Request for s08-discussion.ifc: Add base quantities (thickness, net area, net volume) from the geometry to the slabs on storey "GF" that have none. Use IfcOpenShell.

First a look at what the model holds.

```python
import ifcopenshell
import ifcopenshell.util.element
import ifcopenshell.util.unit

model = ifcopenshell.open("s08-discussion.ifc")
print(model.schema)
for unit_type in ("LENGTHUNIT", "AREAUNIT", "VOLUMEUNIT"):
    print(unit_type, ifcopenshell.util.unit.calculate_unit_scale(model, unit_type))
storey = next(s for s in model.by_type("IfcBuildingStorey") if s.Name == "GF")
slabs = [e for e in ifcopenshell.util.element.get_decomposition(storey) if e.is_a("IfcSlab")]
for e in sorted(slabs, key=lambda e: e.id()):
    print(e.id(), e.is_a(), e.Name, list(ifcopenshell.util.element.get_psets(e, qtos_only=True)), sep=" | ")
```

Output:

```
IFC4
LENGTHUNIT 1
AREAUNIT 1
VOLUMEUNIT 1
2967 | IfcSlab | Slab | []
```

```python
import ifcopenshell
import ifcopenshell.api.pset
import ifcopenshell.geom
import ifcopenshell.util.element
import ifcopenshell.util.shape
import ifcopenshell.util.unit

model = ifcopenshell.open("s08-discussion.ifc")
unit_scale = ifcopenshell.util.unit.calculate_unit_scale(model)
area_scale = ifcopenshell.util.unit.calculate_unit_scale(model, "AREAUNIT")
volume_scale = ifcopenshell.util.unit.calculate_unit_scale(model, "VOLUMEUNIT")
settings = ifcopenshell.geom.settings()

storey = next(s for s in model.by_type("IfcBuildingStorey") if s.Name == "GF")
slabs = [e for e in ifcopenshell.util.element.get_decomposition(storey) if e.is_a("IfcSlab")]

for e in sorted(slabs, key=lambda e: e.id()):
    if ifcopenshell.util.element.get_psets(e, qtos_only=True, should_inherit=False):
        continue
    # Geometry comes back in metres, in the element's own axes.
    shape = ifcopenshell.geom.create_shape(settings, e)
    values = {
        "Width": ifcopenshell.util.shape.get_z(shape.geometry) / unit_scale,
        "NetArea": ifcopenshell.util.shape.get_footprint_area(shape.geometry) / area_scale,
        "NetVolume": ifcopenshell.util.shape.get_volume(shape.geometry) / volume_scale,
    }
    qto = ifcopenshell.api.pset.add_qto(model, product=e, name="Qto_SlabBaseQuantities")
    ifcopenshell.api.pset.edit_qto(model, qto=qto, properties=values)
    print(e.id(), {k: round(v, 3) for k, v in values.items()})

model.write("s08-discussion_edited.ifc")
```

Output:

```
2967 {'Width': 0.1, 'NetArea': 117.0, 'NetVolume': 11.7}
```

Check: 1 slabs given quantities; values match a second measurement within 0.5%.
